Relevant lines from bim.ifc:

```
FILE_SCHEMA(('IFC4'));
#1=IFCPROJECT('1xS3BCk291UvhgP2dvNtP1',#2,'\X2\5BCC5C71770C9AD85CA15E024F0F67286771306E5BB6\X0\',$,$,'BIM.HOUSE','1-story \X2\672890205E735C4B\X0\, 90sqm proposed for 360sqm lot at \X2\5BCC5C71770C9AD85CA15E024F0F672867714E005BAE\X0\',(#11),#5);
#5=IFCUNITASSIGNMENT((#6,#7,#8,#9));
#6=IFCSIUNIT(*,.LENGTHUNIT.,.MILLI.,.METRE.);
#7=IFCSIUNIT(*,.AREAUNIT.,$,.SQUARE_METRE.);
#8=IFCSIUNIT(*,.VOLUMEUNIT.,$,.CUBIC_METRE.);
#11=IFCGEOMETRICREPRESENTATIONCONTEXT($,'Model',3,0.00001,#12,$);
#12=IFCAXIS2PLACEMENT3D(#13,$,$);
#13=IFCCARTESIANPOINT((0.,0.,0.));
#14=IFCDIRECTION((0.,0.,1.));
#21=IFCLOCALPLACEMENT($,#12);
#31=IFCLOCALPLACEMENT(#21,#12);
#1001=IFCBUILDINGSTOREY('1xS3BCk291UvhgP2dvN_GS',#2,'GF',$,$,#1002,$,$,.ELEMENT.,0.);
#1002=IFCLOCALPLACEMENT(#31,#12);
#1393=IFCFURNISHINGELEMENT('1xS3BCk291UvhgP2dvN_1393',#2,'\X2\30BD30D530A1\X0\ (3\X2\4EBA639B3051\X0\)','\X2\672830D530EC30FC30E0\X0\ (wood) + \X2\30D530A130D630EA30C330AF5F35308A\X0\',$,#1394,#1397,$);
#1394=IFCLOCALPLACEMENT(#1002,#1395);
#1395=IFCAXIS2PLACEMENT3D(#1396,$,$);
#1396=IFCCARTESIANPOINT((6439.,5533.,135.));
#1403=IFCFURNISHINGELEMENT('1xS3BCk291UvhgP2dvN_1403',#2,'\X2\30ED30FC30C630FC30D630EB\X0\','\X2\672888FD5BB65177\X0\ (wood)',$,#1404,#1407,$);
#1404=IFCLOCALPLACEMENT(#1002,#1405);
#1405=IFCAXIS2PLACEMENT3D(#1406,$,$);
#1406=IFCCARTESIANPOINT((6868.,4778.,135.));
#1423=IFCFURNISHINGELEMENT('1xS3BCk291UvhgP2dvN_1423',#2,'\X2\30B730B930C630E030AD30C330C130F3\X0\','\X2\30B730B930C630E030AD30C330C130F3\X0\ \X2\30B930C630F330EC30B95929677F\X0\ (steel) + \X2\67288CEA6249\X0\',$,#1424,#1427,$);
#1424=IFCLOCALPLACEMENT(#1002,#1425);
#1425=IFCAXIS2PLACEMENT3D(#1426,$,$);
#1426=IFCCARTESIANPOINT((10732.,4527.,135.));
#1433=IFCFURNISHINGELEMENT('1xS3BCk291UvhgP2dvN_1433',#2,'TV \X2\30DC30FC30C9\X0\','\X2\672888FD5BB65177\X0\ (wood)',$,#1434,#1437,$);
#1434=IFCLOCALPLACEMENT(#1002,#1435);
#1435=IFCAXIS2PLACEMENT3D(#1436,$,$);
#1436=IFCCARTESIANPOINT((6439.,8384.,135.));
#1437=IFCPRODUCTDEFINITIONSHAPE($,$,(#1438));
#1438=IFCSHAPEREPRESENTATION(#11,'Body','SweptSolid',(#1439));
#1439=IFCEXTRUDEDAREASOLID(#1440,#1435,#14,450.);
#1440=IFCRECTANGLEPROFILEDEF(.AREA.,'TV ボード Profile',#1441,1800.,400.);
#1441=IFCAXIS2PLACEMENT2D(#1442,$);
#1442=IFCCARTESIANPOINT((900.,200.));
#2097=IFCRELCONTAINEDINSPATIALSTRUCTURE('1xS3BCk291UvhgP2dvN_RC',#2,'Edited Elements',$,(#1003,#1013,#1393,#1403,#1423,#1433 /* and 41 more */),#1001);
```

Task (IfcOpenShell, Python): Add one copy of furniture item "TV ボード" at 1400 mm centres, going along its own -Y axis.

```python
import ifcopenshell
import ifcopenshell.api.geometry
import ifcopenshell.api.root
import ifcopenshell.util.element
import ifcopenshell.util.placement
import ifcopenshell.util.unit

model = ifcopenshell.open("bim.ifc")
unit_scale = ifcopenshell.util.unit.calculate_unit_scale(model)


def reuse_history(source, copy):
    """copy_class also copies each property set's owner history, people and application; keep the originals."""
    for rel in copy.IsDefinedBy:
        if rel.is_a("IfcRelDefinesByProperties") and (history := rel.RelatingPropertyDefinition.OwnerHistory):
            rel.RelatingPropertyDefinition.OwnerHistory = source.OwnerHistory
            ifcopenshell.util.element.remove_deep2(model, history)


source = model.by_guid("1xS3BCk291UvhgP2dvN_1433")
base = ifcopenshell.util.placement.get_local_placement(source.ObjectPlacement)
step = -base[:3, 1] * 1.4 / unit_scale

for i in range(1, 2):
    copy = ifcopenshell.api.root.copy_class(model, product=source)
    copy.Representation = ifcopenshell.util.element.copy_deep(
        model, source.Representation, exclude=["IfcGeometricRepresentationContext", "IfcRepresentationMap"]
    )
    reuse_history(source, copy)
    matrix = base.copy()
    matrix[:3, 3] += i * step
    print("added at", matrix[:3, 3].round(3) + 0.0)
    ifcopenshell.api.geometry.edit_object_placement(model, product=copy, matrix=matrix, is_si=False)

model.write("bim-out.ifc")
```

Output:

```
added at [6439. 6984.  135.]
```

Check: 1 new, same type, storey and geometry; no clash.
